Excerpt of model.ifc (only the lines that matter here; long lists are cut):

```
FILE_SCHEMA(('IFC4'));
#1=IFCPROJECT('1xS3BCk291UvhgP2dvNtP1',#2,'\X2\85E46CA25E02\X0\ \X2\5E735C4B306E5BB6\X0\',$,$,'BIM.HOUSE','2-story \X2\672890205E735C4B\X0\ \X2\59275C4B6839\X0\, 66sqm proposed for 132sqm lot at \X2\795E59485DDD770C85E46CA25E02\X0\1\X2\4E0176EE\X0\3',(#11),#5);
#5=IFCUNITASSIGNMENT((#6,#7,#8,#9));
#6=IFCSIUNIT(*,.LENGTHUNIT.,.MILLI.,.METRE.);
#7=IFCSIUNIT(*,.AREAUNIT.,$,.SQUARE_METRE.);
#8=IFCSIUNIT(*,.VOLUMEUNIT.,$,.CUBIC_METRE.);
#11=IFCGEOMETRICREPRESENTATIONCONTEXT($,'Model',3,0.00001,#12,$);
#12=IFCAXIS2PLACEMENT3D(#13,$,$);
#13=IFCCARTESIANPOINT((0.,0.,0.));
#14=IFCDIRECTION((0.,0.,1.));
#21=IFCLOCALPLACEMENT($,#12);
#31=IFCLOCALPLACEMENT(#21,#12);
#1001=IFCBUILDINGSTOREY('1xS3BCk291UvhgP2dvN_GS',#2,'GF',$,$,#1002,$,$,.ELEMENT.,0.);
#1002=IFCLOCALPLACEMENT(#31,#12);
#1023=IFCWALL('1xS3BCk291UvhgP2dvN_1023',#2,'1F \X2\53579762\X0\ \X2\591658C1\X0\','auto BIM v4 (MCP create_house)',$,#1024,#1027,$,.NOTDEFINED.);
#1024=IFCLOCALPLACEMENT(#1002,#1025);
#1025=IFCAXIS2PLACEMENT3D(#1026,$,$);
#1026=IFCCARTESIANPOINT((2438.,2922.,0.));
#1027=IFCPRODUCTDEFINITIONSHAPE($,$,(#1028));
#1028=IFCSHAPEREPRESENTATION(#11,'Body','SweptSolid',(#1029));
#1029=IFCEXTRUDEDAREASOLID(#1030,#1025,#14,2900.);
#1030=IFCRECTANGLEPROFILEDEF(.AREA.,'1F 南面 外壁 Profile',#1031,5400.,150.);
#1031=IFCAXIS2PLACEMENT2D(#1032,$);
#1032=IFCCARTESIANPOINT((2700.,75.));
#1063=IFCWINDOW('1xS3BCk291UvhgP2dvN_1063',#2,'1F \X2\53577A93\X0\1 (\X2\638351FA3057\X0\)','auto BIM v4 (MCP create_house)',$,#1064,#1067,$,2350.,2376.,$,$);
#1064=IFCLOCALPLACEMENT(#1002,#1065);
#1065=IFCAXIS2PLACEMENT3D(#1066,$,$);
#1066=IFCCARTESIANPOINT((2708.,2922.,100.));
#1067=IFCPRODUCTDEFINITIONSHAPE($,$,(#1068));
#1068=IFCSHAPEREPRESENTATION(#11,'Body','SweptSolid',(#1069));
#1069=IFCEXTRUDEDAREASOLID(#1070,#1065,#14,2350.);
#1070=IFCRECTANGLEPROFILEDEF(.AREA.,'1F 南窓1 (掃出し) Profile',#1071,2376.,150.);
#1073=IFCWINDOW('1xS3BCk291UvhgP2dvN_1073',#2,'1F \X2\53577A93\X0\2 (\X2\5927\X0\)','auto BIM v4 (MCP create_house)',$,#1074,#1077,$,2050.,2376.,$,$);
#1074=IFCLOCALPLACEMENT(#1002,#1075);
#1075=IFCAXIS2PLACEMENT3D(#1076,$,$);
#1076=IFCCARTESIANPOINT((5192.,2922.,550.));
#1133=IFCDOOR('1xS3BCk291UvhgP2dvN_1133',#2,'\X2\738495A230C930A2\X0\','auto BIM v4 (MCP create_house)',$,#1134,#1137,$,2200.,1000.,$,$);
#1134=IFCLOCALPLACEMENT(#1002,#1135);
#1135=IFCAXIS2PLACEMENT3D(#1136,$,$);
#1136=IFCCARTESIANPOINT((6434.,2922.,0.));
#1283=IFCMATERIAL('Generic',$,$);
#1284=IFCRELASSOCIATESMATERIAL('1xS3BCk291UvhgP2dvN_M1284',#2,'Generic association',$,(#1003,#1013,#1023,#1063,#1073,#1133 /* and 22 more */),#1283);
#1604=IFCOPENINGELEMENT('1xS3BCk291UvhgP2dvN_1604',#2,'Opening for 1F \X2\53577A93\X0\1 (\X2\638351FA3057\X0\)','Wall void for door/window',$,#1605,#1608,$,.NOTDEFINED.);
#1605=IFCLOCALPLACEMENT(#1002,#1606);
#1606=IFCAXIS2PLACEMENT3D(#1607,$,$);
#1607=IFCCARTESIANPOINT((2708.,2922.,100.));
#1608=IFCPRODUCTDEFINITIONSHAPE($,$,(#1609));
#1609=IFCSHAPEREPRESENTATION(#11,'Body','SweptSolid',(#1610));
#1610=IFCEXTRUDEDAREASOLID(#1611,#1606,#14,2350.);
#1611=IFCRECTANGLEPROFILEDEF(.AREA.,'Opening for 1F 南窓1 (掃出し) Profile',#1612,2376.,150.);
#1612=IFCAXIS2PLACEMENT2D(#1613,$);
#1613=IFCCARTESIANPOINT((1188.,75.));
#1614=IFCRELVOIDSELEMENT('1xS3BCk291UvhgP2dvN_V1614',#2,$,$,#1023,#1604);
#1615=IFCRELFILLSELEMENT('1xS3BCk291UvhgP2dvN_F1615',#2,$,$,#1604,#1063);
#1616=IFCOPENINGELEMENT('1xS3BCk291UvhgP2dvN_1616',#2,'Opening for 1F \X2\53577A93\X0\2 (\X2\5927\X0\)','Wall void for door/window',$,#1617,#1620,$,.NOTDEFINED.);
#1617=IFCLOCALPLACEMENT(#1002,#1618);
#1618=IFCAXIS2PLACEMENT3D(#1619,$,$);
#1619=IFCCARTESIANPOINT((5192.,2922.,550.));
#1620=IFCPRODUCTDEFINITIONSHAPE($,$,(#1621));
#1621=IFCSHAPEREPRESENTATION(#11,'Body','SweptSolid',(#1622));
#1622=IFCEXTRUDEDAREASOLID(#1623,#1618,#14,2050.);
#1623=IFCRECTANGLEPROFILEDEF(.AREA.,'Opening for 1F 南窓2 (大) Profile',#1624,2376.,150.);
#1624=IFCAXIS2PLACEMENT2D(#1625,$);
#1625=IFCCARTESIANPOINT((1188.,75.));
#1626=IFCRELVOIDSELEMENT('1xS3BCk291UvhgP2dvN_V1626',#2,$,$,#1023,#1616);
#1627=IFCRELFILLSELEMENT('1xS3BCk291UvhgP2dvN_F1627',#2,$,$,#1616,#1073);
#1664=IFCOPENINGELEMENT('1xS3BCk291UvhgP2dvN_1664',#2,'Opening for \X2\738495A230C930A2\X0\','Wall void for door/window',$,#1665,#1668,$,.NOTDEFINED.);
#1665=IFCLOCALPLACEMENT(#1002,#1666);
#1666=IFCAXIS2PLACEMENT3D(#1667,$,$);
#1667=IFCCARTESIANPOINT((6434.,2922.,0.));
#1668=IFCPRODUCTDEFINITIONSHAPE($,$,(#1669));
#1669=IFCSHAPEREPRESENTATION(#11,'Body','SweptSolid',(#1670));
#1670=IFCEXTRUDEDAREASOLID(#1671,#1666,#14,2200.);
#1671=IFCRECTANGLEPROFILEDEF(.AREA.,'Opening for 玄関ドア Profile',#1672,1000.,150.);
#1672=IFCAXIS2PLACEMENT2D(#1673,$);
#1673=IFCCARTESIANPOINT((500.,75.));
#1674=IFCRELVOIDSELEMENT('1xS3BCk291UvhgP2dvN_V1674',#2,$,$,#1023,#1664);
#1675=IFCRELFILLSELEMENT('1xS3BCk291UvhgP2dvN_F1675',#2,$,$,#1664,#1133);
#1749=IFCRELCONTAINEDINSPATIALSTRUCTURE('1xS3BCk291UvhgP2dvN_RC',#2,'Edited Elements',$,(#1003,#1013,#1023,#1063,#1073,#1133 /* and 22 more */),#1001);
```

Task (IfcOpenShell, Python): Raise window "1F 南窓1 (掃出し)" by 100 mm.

```python
import numpy as np
import ifcopenshell
import ifcopenshell.api.geometry
import ifcopenshell.util.placement
import ifcopenshell.util.unit

model = ifcopenshell.open("model.ifc")
unit_scale = ifcopenshell.util.unit.calculate_unit_scale(model)

window = model.by_id(1063)
opening = window.FillsVoids[0].RelatingOpeningElement
dz = 100.0

shift = np.array([0.0, 0.0, dz])
# The window is not placed relative to its opening, so move both.
for product in (opening, window):
    matrix = ifcopenshell.util.placement.get_local_placement(product.ObjectPlacement)
    matrix[:3, 3] += shift
    ifcopenshell.api.geometry.edit_object_placement(model, product=product, matrix=matrix, is_si=False)

print(f"moved by {dz * unit_scale:+.3f} m")

model.write("model_v2.ifc")
```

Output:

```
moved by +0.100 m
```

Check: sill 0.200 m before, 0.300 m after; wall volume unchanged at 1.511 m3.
